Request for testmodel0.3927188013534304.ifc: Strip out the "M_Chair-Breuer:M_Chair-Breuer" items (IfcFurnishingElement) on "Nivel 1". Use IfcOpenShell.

First a look at what the model holds.

```python
import ifcopenshell
import ifcopenshell.util.element

model = ifcopenshell.open("testmodel0.3927188013534304.ifc")
print(model.schema)
storey = next(s for s in model.by_type("IfcBuildingStorey") if s.Name == "Nivel 1")
furniture = [e for e in ifcopenshell.util.element.get_decomposition(storey) if e.is_a("IfcFurnishingElement")]
seen = {}
for e in furniture:
    element_type = ifcopenshell.util.element.get_type(e)
    name = element_type.Name if element_type not in (None, e) else None
    seen[name] = seen.get(name, 0) + 1
for name, count in sorted(seen.items(), key=str):
    print(count, "x", name)
```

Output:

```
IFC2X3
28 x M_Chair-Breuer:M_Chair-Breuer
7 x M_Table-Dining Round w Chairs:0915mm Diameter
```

```python
import ifcopenshell
import ifcopenshell.api.root
import ifcopenshell.util.element

model = ifcopenshell.open("testmodel0.3927188013534304.ifc")

storey = next(s for s in model.by_type("IfcBuildingStorey") if s.Name == "Nivel 1")
furniture = [e for e in ifcopenshell.util.element.get_decomposition(storey) if e.is_a("IfcFurnishingElement")]
targets = [e for e in furniture if (t := ifcopenshell.util.element.get_type(e)) not in (None, e) and t.Name == "M_Chair-Breuer:M_Chair-Breuer"]

for e in targets:
    ifcopenshell.api.root.remove_product(model, product=e)
print(len(targets), "removed")

model.write("testmodel0.3927188013534304-out.ifc")
```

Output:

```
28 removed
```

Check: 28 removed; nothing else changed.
